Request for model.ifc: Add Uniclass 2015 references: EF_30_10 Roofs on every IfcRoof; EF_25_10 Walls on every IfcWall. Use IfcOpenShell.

First a look at what the model holds.

```python
import ifcopenshell

model = ifcopenshell.open("model.ifc")
print(model.schema)
print("classifications:", [c.Name for c in model.by_type("IfcClassification")])
for ifc_class in ("IfcDoor", "IfcRoof", "IfcStair", "IfcWall", "IfcWindow"):
    print(ifc_class, len(model.by_type(ifc_class)))
```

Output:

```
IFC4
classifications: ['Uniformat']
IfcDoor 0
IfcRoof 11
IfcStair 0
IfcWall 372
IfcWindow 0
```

```python
import ifcopenshell
import ifcopenshell.api.classification

model = ifcopenshell.open("model.ifc")

system = ifcopenshell.api.classification.add_classification(model, classification="Uniclass 2015")

codes = {
    "IfcRoof": ("EF_30_10", "Roofs"),
    "IfcWall": ("EF_25_10", "Walls"),
}
for ifc_class, (code, name) in codes.items():
    products = model.by_type(ifc_class)
    ifcopenshell.api.classification.add_reference(
        model, products=products, classification=system, identification=code, name=name
    )
    print(code, len(products))

model.write("model_edited.ifc")
```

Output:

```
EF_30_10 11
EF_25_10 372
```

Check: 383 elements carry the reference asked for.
